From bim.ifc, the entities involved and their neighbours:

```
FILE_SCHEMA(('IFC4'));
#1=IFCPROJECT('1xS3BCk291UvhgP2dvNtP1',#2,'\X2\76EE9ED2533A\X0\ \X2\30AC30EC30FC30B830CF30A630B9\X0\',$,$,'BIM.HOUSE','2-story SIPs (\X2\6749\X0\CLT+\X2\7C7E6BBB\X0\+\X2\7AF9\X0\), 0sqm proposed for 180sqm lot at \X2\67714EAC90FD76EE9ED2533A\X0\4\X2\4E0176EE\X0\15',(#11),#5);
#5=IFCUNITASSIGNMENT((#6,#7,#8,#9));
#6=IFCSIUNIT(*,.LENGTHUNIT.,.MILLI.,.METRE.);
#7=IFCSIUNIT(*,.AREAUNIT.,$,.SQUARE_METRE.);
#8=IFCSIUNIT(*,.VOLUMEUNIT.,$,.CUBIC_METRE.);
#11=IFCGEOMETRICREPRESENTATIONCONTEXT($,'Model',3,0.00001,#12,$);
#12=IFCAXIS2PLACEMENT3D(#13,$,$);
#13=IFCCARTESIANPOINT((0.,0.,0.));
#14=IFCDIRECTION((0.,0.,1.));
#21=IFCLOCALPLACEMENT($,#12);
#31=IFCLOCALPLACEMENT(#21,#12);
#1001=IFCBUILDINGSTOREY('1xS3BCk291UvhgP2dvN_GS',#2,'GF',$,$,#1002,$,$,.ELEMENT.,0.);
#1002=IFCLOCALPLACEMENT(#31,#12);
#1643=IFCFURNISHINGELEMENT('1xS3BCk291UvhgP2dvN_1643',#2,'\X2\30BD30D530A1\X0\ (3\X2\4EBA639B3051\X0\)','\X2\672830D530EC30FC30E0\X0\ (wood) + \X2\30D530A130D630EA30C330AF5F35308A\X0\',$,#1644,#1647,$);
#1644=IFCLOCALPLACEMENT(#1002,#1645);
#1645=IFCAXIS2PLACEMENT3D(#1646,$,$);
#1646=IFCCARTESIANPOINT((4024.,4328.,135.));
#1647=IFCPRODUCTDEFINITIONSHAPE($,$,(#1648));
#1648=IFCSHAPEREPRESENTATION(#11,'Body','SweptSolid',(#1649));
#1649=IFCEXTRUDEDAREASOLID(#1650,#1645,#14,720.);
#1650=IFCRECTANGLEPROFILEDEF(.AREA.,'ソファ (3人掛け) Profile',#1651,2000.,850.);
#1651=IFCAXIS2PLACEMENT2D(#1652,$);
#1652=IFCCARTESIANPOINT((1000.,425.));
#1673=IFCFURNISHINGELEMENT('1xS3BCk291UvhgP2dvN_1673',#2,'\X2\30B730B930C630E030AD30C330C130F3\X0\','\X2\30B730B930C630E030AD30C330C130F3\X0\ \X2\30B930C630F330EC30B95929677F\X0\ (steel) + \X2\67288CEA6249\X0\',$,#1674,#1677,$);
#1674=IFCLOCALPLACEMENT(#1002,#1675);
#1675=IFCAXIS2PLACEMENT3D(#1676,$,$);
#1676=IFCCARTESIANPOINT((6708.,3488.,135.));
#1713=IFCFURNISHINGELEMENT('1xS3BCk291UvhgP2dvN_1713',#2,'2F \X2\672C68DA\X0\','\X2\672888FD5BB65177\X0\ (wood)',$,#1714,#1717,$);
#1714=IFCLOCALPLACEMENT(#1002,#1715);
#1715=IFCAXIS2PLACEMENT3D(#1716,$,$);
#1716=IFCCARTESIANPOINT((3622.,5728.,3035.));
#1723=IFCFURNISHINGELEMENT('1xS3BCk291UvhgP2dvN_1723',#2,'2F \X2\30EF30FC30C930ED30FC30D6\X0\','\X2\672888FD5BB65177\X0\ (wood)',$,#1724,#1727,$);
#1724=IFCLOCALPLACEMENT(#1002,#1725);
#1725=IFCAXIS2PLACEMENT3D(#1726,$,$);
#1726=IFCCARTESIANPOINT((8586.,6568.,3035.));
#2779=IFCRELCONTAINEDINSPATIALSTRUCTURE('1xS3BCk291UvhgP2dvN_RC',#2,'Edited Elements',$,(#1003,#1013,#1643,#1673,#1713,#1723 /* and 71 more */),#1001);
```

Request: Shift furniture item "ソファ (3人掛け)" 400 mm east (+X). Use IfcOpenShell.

```python
import ifcopenshell
import ifcopenshell.api.geometry
import ifcopenshell.util.placement

model = ifcopenshell.open("bim.ifc")

item = model.by_guid("1xS3BCk291UvhgP2dvN_1643")
matrix = ifcopenshell.util.placement.get_local_placement(item.ObjectPlacement)
matrix[0, 3] += 400.0
ifcopenshell.api.geometry.edit_object_placement(model, product=item, matrix=matrix, is_si=False)

print(ifcopenshell.util.placement.get_local_placement(item.ObjectPlacement).round(3) + 0.0)

model.write("bim-out.ifc")
```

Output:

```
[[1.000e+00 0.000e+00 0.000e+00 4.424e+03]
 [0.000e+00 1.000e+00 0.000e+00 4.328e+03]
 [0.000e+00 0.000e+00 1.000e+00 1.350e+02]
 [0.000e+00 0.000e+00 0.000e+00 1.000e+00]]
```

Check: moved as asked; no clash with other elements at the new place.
